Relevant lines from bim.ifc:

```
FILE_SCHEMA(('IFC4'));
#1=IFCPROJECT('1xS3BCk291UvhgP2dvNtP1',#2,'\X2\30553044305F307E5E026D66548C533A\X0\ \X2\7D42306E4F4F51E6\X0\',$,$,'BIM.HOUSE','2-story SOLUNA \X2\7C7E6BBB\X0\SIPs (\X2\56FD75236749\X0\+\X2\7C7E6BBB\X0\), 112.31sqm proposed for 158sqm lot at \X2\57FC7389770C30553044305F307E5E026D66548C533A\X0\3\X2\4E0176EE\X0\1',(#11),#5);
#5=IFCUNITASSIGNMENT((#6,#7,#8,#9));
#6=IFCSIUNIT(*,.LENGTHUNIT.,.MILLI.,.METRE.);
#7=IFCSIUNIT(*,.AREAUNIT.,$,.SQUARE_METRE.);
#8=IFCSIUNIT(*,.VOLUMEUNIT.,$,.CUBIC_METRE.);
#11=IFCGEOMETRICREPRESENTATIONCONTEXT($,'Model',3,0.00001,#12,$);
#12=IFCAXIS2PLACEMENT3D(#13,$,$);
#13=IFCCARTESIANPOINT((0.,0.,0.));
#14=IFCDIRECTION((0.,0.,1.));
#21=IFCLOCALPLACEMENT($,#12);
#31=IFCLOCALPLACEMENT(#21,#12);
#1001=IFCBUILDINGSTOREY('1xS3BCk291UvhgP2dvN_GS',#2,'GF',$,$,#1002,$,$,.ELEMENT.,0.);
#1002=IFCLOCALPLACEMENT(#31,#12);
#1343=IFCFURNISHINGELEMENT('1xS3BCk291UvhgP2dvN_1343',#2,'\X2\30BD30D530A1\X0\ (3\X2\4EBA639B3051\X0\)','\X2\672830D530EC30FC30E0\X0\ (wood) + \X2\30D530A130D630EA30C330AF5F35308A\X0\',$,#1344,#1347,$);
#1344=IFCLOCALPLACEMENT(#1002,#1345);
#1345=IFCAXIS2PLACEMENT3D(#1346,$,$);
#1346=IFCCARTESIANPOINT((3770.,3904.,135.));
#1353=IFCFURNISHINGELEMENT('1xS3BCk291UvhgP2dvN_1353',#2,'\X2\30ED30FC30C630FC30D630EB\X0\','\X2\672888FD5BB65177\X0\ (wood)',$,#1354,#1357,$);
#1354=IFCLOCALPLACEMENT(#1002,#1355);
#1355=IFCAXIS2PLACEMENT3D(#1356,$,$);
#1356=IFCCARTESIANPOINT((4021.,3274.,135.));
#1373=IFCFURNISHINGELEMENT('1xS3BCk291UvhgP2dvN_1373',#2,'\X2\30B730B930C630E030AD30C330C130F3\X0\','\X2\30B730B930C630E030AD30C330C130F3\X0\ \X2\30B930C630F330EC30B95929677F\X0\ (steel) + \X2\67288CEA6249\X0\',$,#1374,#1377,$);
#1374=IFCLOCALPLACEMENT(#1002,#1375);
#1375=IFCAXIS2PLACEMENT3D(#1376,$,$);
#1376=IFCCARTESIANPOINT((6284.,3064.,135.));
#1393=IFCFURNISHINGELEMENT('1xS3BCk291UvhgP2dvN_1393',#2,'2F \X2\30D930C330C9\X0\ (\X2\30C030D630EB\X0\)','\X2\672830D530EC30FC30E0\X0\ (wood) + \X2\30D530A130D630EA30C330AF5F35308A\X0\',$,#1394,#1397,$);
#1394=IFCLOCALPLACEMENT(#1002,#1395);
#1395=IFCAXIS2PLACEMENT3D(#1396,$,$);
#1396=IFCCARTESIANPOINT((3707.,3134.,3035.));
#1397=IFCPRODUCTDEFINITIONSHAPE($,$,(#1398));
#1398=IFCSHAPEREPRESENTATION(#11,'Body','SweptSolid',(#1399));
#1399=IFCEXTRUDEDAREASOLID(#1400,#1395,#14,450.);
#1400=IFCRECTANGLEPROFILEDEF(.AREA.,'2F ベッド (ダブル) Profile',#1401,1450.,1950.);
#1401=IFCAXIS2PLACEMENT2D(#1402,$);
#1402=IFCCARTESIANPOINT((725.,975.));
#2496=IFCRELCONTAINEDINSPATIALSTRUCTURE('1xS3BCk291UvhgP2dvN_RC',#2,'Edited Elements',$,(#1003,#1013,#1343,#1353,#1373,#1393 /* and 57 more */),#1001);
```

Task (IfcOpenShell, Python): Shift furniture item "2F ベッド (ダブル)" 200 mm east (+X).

```python
import ifcopenshell
import ifcopenshell.api.geometry
import ifcopenshell.util.placement
import ifcopenshell.util.unit

model = ifcopenshell.open("bim.ifc")
unit_scale = ifcopenshell.util.unit.calculate_unit_scale(model)

item = model.by_guid("1xS3BCk291UvhgP2dvN_1393")
matrix = ifcopenshell.util.placement.get_local_placement(item.ObjectPlacement)
matrix[0, 3] += 0.2 / unit_scale
ifcopenshell.api.geometry.edit_object_placement(model, product=item, matrix=matrix, is_si=False)

print(ifcopenshell.util.placement.get_local_placement(item.ObjectPlacement).round(3) + 0.0)

model.write("bim_v2.ifc")
```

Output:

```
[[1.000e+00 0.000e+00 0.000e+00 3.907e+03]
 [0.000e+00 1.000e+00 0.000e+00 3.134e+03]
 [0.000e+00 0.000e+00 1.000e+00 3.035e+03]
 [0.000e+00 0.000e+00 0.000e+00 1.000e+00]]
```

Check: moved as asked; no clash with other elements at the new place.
